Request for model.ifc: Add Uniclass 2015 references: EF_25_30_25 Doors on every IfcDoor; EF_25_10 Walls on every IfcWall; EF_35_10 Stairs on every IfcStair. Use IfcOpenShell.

First a look at what the model holds.

```python
import ifcopenshell

model = ifcopenshell.open("model.ifc")
print(model.schema)
print("classifications:", [c.Name for c in model.by_type("IfcClassification")])
for ifc_class in ("IfcDoor", "IfcRoof", "IfcStair", "IfcWall", "IfcWindow"):
    print(ifc_class, len(model.by_type(ifc_class)))
```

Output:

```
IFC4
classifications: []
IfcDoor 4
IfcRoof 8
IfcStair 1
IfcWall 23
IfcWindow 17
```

```python
import ifcopenshell
import ifcopenshell.api.classification

model = ifcopenshell.open("model.ifc")

system = ifcopenshell.api.classification.add_classification(model, classification="Uniclass 2015")

codes = {
    "IfcDoor": ("EF_25_30_25", "Doors"),
    "IfcWall": ("EF_25_10", "Walls"),
    "IfcStair": ("EF_35_10", "Stairs"),
}
for ifc_class, (code, name) in codes.items():
    products = model.by_type(ifc_class)
    ifcopenshell.api.classification.add_reference(
        model, products=products, classification=system, identification=code, name=name
    )
    print(code, len(products))

model.write("model-out.ifc")
```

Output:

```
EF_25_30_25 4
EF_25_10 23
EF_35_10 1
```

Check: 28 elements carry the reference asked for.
